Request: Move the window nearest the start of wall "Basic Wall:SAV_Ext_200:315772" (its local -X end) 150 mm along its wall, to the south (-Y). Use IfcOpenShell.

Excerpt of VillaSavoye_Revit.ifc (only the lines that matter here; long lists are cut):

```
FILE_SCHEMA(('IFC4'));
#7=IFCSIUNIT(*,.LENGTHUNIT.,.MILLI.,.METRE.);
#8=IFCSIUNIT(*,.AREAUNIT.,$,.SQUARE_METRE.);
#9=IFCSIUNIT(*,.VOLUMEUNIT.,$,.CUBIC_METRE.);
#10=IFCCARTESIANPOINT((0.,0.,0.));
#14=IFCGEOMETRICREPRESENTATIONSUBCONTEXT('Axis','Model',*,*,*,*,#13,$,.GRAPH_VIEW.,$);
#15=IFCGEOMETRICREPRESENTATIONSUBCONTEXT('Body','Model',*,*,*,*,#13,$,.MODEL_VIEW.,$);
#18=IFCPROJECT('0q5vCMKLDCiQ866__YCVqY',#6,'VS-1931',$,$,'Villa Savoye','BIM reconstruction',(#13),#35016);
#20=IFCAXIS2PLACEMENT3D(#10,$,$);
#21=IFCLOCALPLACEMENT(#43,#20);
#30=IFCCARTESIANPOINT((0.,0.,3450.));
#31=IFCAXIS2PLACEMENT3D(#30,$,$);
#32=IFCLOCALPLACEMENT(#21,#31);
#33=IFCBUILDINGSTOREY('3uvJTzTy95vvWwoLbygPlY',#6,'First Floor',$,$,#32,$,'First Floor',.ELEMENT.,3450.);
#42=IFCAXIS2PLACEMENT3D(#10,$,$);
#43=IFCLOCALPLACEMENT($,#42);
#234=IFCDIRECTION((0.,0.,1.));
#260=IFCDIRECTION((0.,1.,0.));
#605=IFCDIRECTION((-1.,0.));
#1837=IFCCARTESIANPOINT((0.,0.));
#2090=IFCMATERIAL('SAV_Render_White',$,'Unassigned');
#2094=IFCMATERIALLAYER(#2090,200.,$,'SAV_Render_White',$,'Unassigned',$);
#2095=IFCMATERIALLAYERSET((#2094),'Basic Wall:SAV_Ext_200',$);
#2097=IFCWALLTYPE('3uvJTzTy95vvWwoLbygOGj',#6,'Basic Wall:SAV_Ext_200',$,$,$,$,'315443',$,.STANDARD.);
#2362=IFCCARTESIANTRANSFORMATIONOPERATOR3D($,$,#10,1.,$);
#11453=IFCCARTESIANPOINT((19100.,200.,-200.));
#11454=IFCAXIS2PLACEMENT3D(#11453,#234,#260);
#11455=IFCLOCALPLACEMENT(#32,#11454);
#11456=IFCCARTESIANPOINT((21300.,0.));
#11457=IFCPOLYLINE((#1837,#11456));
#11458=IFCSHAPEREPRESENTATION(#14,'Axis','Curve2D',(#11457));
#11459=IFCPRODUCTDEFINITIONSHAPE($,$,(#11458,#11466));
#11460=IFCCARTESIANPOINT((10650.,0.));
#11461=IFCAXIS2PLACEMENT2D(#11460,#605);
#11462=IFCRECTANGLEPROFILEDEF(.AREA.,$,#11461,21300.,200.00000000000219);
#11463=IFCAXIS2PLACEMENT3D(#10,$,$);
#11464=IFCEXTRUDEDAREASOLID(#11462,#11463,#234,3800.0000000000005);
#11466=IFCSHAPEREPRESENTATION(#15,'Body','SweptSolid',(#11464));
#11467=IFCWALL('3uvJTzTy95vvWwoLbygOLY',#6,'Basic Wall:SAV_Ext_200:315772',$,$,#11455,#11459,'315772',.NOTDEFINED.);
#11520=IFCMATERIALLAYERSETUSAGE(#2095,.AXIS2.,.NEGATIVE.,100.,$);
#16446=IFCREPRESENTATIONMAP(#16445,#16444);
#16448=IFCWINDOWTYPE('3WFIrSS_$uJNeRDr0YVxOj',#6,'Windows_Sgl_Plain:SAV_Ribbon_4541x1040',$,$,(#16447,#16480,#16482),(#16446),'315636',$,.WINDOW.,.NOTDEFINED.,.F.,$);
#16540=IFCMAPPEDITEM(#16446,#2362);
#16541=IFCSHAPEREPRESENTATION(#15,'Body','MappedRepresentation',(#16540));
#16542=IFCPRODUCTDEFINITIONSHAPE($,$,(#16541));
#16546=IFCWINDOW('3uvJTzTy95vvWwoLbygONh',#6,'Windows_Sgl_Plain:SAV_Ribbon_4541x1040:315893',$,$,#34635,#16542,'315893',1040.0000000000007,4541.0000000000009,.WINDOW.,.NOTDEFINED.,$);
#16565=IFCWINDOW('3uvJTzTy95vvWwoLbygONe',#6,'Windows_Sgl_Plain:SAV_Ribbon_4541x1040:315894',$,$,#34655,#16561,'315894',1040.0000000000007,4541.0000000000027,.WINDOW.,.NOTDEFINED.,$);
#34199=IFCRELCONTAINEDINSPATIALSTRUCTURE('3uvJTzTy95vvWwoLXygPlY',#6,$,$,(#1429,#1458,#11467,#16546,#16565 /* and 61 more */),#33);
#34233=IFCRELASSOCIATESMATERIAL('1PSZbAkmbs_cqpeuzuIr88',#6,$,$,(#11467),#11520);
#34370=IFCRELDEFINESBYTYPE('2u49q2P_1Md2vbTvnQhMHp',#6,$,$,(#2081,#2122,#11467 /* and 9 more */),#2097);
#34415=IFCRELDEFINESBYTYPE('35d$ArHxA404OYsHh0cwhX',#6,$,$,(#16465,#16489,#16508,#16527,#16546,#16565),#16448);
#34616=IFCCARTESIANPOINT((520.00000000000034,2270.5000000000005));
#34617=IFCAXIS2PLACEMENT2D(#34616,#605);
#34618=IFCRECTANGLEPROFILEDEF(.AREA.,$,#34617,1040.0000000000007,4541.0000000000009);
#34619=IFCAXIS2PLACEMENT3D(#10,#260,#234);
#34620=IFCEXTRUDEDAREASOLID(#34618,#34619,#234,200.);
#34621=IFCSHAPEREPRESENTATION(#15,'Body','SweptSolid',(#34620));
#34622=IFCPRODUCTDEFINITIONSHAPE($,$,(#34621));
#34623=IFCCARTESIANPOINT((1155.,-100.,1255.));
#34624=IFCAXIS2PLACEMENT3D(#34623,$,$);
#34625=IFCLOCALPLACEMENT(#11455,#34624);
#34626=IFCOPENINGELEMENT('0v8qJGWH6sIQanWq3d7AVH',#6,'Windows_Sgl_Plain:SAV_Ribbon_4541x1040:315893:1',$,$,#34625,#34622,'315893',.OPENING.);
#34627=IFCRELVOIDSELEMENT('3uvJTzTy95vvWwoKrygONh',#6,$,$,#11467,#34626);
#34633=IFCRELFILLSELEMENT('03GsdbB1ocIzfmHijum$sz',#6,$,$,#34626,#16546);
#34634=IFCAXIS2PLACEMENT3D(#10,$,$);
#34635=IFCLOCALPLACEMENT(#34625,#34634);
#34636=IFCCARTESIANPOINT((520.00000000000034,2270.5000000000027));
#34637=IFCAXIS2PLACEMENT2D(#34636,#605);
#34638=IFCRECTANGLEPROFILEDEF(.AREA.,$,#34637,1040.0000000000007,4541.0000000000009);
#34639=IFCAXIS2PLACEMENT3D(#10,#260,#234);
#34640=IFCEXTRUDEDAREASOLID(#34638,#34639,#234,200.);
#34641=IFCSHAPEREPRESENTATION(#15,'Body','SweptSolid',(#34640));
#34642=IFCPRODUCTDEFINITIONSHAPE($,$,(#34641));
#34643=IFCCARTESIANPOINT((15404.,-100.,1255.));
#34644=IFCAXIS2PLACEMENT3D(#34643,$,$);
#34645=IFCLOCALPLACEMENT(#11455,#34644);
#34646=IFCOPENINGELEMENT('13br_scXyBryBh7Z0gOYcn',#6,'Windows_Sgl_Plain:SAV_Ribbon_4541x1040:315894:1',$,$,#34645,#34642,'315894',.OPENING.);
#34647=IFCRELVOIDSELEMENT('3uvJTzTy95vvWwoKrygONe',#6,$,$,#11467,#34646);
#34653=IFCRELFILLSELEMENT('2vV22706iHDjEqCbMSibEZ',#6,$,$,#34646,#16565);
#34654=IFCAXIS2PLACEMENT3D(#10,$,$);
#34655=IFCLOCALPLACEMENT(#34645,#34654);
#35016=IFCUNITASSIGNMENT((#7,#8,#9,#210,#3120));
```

```python
import ifcopenshell
import ifcopenshell.api.geometry
import ifcopenshell.util.placement
import ifcopenshell.util.unit

model = ifcopenshell.open("VillaSavoye_Revit.ifc")
unit_scale = ifcopenshell.util.unit.calculate_unit_scale(model)

window = model.by_id(16546)
opening = window.FillsVoids[0].RelatingOpeningElement
wall = opening.VoidsElements[0].RelatingBuildingElement

wall_matrix = ifcopenshell.util.placement.get_local_placement(wall.ObjectPlacement)
shift = wall_matrix[:3, 0] * -0.15 / unit_scale
before = ifcopenshell.util.placement.get_local_placement(window.ObjectPlacement)[:3, 3].copy()

# The window is placed relative to its opening, so it follows when the opening moves.
matrix = ifcopenshell.util.placement.get_local_placement(opening.ObjectPlacement)
matrix[:3, 3] += shift
ifcopenshell.api.geometry.edit_object_placement(
    model, product=opening, matrix=matrix, is_si=False, should_transform_children=True
)

after = ifcopenshell.util.placement.get_local_placement(window.ObjectPlacement)[:3, 3]
print("window moved by", (after - before).round(3) + 0.0)

model.write("VillaSavoye_Revit_edited.ifc")
```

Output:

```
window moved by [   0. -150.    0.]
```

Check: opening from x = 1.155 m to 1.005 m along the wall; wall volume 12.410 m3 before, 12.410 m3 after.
